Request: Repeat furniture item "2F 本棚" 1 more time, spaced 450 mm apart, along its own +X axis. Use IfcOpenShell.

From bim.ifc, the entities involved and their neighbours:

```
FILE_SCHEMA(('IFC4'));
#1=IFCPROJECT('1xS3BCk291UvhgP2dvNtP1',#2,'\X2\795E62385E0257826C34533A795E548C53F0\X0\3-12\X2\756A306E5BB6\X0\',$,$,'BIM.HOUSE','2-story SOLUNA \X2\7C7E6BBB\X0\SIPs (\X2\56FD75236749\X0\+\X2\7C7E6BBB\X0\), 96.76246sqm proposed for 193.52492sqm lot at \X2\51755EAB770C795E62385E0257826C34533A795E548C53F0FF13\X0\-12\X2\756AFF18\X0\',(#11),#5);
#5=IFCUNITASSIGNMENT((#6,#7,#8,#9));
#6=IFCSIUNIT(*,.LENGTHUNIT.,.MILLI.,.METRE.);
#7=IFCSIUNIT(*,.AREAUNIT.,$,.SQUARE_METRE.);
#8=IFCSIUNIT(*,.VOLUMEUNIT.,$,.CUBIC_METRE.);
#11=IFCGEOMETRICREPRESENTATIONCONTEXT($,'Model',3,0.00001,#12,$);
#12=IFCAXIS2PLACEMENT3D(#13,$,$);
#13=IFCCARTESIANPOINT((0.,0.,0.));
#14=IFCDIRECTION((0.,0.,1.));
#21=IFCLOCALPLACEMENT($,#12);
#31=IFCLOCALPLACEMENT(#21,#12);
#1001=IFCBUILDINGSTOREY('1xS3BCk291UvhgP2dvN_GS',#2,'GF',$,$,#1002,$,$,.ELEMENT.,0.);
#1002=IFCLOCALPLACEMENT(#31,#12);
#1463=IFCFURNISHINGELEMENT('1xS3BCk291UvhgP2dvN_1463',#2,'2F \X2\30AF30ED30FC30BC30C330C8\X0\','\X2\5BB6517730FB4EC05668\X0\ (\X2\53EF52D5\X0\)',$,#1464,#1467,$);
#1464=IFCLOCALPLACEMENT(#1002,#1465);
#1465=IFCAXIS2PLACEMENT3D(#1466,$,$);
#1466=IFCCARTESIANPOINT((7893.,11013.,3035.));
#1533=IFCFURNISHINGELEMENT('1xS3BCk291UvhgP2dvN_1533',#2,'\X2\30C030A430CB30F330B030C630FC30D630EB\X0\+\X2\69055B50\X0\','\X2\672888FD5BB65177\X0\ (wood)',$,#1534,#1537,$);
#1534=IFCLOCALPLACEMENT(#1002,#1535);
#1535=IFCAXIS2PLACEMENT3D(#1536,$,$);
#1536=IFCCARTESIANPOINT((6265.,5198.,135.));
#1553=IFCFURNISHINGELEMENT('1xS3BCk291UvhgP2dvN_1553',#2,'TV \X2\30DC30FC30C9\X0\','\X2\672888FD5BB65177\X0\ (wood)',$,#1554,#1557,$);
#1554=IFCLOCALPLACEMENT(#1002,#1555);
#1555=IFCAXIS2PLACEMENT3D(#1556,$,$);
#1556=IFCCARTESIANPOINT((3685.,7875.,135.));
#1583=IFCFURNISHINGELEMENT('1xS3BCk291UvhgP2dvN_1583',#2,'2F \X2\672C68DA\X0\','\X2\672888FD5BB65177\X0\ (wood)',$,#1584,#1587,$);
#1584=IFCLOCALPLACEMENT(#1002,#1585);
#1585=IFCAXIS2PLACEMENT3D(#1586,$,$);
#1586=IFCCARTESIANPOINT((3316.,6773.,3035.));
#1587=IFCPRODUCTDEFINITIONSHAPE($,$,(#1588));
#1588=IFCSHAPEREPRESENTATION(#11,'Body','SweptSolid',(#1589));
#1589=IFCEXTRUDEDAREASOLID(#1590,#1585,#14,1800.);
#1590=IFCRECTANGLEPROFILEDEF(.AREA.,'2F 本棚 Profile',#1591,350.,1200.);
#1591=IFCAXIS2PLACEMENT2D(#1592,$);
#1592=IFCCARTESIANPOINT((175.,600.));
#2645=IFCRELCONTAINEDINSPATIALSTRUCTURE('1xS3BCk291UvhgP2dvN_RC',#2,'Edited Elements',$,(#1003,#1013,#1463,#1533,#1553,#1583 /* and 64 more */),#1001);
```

```python
import ifcopenshell
import ifcopenshell.api.geometry
import ifcopenshell.api.root
import ifcopenshell.util.element
import ifcopenshell.util.placement

model = ifcopenshell.open("bim.ifc")


def reuse_history(source, copy):
    """copy_class also copies each property set's owner history, people and application; keep the originals."""
    for rel in copy.IsDefinedBy:
        if rel.is_a("IfcRelDefinesByProperties") and (history := rel.RelatingPropertyDefinition.OwnerHistory):
            rel.RelatingPropertyDefinition.OwnerHistory = source.OwnerHistory
            ifcopenshell.util.element.remove_deep2(model, history)


source = model.by_guid("1xS3BCk291UvhgP2dvN_1583")
base = ifcopenshell.util.placement.get_local_placement(source.ObjectPlacement)
step = base[:3, 0] * 450.0

for i in range(1, 2):
    copy = ifcopenshell.api.root.copy_class(model, product=source)
    copy.Representation = ifcopenshell.util.element.copy_deep(
        model, source.Representation, exclude=["IfcGeometricRepresentationContext", "IfcRepresentationMap"]
    )
    reuse_history(source, copy)
    matrix = base.copy()
    matrix[:3, 3] += i * step
    print("added at", matrix[:3, 3].round(3) + 0.0)
    ifcopenshell.api.geometry.edit_object_placement(model, product=copy, matrix=matrix, is_si=False)

model.write("bim-out.ifc")
```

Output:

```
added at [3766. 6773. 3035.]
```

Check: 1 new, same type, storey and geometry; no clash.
